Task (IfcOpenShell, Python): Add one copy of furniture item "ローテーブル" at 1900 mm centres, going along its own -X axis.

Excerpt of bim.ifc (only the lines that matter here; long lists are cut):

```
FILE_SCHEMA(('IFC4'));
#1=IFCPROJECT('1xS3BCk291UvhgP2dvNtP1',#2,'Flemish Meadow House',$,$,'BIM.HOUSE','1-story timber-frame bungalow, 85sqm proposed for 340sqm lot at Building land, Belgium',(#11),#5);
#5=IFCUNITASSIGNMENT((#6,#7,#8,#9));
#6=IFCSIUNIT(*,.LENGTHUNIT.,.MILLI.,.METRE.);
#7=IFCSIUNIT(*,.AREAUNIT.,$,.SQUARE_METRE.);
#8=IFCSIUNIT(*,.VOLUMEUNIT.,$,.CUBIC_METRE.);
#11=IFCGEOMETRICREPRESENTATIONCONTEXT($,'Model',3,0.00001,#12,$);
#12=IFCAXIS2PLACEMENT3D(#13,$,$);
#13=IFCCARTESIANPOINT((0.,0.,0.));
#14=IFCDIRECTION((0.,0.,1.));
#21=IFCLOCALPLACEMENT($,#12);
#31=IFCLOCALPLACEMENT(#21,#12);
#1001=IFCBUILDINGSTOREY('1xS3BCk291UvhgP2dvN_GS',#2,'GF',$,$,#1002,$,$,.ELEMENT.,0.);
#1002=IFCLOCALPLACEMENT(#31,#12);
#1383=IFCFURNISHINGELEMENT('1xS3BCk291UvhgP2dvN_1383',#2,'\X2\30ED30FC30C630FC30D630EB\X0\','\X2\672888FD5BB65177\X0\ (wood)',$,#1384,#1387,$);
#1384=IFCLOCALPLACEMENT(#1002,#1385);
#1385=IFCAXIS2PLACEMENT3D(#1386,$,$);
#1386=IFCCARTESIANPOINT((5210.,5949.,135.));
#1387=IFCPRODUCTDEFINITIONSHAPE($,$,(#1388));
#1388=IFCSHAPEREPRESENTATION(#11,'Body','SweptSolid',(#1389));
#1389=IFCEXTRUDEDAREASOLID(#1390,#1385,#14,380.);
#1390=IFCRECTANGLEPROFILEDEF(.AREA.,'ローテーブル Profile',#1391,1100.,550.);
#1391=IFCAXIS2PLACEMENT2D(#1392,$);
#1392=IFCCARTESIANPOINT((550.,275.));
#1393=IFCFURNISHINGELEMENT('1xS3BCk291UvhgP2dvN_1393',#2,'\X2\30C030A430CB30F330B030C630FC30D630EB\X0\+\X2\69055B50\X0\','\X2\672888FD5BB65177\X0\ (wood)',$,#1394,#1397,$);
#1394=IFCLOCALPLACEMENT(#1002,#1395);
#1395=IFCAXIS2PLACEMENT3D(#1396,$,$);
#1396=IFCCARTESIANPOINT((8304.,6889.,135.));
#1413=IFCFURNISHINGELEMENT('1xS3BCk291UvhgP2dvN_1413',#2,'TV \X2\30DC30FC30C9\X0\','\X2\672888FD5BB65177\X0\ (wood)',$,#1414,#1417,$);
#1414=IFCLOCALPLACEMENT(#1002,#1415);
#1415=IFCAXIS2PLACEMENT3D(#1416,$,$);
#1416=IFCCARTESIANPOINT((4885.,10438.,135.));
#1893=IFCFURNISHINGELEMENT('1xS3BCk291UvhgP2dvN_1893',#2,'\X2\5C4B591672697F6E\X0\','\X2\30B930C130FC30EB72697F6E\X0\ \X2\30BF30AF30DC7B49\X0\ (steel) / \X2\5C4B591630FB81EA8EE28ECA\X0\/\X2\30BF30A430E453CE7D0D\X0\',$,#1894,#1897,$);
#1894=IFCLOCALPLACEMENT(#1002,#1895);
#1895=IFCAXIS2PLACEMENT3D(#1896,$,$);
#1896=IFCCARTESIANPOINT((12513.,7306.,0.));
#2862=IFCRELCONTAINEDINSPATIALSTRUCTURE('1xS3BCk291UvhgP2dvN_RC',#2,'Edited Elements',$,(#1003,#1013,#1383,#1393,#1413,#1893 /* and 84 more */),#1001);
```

```python
import ifcopenshell
import ifcopenshell.api.geometry
import ifcopenshell.api.root
import ifcopenshell.util.element
import ifcopenshell.util.placement

model = ifcopenshell.open("bim.ifc")


def reuse_history(source, copy):
    """copy_class also copies each property set's owner history, people and application; keep the originals."""
    for rel in copy.IsDefinedBy:
        if rel.is_a("IfcRelDefinesByProperties") and (history := rel.RelatingPropertyDefinition.OwnerHistory):
            rel.RelatingPropertyDefinition.OwnerHistory = source.OwnerHistory
            ifcopenshell.util.element.remove_deep2(model, history)


source = model.by_id(1383)
base = ifcopenshell.util.placement.get_local_placement(source.ObjectPlacement)
step = -base[:3, 0] * 1900.0

for i in range(1, 2):
    copy = ifcopenshell.api.root.copy_class(model, product=source)
    copy.Representation = ifcopenshell.util.element.copy_deep(
        model, source.Representation, exclude=["IfcGeometricRepresentationContext", "IfcRepresentationMap"]
    )
    reuse_history(source, copy)
    matrix = base.copy()
    matrix[:3, 3] += i * step
    print("added at", matrix[:3, 3].round(3) + 0.0)
    ifcopenshell.api.geometry.edit_object_placement(model, product=copy, matrix=matrix, is_si=False)

model.write("bim_v2.ifc")
```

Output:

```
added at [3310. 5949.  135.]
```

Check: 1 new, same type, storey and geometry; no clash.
